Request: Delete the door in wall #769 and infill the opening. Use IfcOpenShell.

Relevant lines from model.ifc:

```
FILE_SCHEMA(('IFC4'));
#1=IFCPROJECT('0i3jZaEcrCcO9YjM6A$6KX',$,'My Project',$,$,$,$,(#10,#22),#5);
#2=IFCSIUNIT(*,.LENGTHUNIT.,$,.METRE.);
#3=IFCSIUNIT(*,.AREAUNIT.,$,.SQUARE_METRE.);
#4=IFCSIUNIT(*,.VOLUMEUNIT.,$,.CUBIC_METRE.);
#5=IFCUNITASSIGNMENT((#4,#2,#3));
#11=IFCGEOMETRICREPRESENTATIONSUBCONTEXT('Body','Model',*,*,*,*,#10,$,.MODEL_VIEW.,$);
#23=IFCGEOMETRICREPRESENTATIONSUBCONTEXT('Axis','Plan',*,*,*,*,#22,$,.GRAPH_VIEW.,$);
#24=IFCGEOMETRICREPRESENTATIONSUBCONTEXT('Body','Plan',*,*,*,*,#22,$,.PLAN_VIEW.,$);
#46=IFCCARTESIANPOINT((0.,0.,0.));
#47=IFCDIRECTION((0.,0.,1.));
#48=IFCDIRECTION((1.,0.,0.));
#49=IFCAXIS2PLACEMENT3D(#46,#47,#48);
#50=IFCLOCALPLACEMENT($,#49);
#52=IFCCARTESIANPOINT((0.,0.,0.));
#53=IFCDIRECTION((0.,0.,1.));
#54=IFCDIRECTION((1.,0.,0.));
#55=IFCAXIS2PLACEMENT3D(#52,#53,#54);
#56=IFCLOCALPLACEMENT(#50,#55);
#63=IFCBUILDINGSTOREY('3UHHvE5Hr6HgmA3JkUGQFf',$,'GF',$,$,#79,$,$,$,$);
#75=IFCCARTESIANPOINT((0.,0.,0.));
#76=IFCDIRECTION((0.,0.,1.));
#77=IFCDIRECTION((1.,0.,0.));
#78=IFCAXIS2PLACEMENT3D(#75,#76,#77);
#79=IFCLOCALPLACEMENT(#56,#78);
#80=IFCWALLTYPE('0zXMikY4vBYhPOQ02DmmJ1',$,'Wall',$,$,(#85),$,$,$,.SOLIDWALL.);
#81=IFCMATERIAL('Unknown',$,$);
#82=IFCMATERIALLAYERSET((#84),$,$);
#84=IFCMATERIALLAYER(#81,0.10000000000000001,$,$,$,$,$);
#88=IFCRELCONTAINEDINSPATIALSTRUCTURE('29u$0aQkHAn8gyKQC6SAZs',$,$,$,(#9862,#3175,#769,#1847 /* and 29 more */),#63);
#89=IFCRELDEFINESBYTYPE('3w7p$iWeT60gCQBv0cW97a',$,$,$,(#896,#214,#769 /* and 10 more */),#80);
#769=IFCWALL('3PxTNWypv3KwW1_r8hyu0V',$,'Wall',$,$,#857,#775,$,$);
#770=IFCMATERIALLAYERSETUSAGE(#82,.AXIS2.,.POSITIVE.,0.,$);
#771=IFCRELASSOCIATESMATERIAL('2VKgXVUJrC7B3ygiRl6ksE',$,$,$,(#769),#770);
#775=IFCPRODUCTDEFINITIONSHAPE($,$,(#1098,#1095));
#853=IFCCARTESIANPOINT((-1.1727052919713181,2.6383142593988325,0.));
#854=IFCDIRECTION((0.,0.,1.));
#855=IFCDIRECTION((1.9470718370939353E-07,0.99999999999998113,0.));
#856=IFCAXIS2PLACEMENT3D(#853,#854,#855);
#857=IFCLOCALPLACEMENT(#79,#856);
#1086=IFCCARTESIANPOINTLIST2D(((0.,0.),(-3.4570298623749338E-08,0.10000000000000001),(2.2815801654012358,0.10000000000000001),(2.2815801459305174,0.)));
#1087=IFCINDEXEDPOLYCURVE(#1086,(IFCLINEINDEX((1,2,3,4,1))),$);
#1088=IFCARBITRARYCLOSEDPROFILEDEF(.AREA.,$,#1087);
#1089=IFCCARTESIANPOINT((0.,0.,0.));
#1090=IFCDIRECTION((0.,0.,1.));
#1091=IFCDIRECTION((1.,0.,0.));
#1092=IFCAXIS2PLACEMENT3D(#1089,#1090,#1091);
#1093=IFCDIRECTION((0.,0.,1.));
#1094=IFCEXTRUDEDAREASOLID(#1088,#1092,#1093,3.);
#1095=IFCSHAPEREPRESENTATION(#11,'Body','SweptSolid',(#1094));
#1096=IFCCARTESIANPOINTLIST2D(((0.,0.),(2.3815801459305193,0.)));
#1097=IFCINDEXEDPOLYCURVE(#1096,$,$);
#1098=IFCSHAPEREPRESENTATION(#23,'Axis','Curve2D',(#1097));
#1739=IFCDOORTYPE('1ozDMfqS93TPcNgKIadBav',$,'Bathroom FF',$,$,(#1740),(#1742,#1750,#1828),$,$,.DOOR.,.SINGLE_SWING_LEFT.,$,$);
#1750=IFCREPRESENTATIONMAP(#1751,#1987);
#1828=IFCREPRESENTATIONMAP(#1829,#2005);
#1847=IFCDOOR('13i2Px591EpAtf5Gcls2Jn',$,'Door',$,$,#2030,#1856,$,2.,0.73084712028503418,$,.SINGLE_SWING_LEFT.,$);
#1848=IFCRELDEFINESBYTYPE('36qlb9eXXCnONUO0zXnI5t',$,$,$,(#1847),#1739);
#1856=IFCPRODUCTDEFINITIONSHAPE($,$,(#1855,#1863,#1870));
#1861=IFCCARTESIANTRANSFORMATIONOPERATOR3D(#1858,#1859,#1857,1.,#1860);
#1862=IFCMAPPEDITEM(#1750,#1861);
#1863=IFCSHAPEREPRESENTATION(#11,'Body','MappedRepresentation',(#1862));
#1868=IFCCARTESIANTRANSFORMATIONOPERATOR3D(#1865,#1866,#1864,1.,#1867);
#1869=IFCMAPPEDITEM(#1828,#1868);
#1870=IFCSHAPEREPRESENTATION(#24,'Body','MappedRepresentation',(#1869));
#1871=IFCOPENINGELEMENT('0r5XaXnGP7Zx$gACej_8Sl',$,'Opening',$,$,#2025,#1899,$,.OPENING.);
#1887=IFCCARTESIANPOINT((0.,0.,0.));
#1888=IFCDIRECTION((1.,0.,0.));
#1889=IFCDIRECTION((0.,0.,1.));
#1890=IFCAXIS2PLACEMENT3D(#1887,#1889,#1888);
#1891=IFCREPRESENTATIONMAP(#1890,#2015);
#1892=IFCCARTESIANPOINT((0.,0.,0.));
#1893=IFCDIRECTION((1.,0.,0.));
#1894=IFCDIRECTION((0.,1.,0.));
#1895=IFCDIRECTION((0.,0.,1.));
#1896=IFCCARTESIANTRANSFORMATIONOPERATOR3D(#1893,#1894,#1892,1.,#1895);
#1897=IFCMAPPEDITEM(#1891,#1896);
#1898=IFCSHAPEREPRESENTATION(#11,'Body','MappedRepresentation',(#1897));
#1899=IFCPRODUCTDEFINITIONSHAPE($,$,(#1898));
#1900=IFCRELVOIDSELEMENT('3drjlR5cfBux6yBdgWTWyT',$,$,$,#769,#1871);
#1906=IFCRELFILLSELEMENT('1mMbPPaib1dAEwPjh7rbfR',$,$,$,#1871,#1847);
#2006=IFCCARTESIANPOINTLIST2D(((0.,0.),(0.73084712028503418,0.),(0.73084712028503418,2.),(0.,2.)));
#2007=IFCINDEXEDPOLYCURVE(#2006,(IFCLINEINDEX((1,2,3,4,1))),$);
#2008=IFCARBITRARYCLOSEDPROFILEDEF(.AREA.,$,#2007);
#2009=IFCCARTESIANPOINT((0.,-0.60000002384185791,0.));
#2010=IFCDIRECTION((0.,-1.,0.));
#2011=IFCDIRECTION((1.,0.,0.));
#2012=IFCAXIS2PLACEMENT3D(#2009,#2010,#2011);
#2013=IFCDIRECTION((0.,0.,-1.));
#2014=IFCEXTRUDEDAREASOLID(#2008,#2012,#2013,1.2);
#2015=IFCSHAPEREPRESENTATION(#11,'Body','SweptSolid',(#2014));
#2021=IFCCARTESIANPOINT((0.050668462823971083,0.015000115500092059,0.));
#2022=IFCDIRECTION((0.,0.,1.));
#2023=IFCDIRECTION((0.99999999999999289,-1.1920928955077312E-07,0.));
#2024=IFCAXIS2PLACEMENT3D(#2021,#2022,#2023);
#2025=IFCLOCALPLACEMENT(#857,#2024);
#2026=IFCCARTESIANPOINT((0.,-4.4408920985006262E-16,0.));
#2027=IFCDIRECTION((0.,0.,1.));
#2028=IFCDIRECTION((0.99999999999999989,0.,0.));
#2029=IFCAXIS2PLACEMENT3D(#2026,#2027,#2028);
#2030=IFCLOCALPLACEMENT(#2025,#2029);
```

```python
import ifcopenshell
import ifcopenshell.api.feature
import ifcopenshell.api.root
import ifcopenshell.geom
import ifcopenshell.util.shape

model = ifcopenshell.open("model.ifc")
settings = ifcopenshell.geom.settings()


def volume(element):
    """Net volume in cubic metres, openings subtracted."""
    shape = ifcopenshell.geom.create_shape(settings, element)
    return ifcopenshell.util.shape.get_volume(shape.geometry)


door = model.by_guid("13i2Px591EpAtf5Gcls2Jn")
opening = door.FillsVoids[0].RelatingOpeningElement
wall = opening.VoidsElements[0].RelatingBuildingElement
before = volume(wall)

ifcopenshell.api.root.remove_product(model, product=door)
ifcopenshell.api.feature.remove_feature(model, feature=opening)

after = volume(wall)

print(f"wall volume {before:.3f} -> {after:.3f} m3")

model.write("model_v2.ifc")
```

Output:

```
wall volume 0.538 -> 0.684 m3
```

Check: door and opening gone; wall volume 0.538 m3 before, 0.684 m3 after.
